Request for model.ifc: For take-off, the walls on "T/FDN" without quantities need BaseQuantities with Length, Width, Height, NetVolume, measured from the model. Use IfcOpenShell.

First a look at what the model holds.

```python
import ifcopenshell
import ifcopenshell.util.element
import ifcopenshell.util.unit

model = ifcopenshell.open("model.ifc")
print(model.schema)
for unit_type in ("LENGTHUNIT", "AREAUNIT", "VOLUMEUNIT"):
    print(unit_type, ifcopenshell.util.unit.calculate_unit_scale(model, unit_type))
storey = next(s for s in model.by_type("IfcBuildingStorey") if s.Name == "T/FDN")
walls = [e for e in ifcopenshell.util.element.get_decomposition(storey) if e.is_a("IfcWall")]
for e in sorted(walls, key=lambda e: e.id()):
    print(e.id(), e.is_a(), e.Name, list(ifcopenshell.util.element.get_psets(e, qtos_only=True)), sep=" | ")
```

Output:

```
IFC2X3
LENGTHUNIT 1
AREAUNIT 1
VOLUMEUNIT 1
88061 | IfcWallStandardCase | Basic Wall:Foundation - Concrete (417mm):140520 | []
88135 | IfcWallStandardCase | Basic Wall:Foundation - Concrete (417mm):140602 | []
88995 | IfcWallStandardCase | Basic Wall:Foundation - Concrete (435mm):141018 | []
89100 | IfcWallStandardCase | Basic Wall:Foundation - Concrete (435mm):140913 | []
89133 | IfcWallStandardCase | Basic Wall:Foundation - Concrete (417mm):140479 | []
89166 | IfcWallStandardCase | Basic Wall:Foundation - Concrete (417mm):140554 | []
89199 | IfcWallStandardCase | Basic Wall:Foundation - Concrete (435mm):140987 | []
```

```python
import ifcopenshell
import ifcopenshell.api.pset
import ifcopenshell.geom
import ifcopenshell.util.element
import ifcopenshell.util.shape
import ifcopenshell.util.unit

model = ifcopenshell.open("model.ifc")
unit_scale = ifcopenshell.util.unit.calculate_unit_scale(model)
volume_scale = ifcopenshell.util.unit.calculate_unit_scale(model, "VOLUMEUNIT")
settings = ifcopenshell.geom.settings()

storey = next(s for s in model.by_type("IfcBuildingStorey") if s.Name == "T/FDN")
walls = [e for e in ifcopenshell.util.element.get_decomposition(storey) if e.is_a("IfcWall")]

for e in sorted(walls, key=lambda e: e.id()):
    if ifcopenshell.util.element.get_psets(e, qtos_only=True, should_inherit=False):
        continue
    # Geometry comes back in metres, in the element's own axes.
    shape = ifcopenshell.geom.create_shape(settings, e)
    values = {
        "Length": ifcopenshell.util.shape.get_x(shape.geometry) / unit_scale,
        "Width": ifcopenshell.util.shape.get_y(shape.geometry) / unit_scale,
        "Height": ifcopenshell.util.shape.get_z(shape.geometry) / unit_scale,
        "NetVolume": ifcopenshell.util.shape.get_volume(shape.geometry) / volume_scale,
    }
    qto = ifcopenshell.api.pset.add_qto(model, product=e, name="BaseQuantities")
    ifcopenshell.api.pset.edit_qto(model, qto=qto, properties=values)
    print(e.id(), {k: round(v, 3) for k, v in values.items()})

model.write("model-out.ifc")
```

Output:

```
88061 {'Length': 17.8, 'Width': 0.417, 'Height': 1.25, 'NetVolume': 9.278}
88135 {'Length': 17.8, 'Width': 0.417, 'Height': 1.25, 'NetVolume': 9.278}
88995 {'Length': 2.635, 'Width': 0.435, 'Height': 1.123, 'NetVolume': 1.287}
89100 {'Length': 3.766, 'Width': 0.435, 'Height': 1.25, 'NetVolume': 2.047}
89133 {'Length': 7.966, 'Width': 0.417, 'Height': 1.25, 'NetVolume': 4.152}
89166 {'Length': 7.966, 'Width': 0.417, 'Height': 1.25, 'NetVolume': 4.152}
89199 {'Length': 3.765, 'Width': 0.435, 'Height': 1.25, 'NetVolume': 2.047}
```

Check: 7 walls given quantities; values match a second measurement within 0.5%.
